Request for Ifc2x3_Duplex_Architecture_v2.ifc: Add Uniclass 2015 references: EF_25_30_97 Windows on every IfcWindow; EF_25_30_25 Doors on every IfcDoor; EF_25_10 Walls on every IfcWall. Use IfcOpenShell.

First a look at what the model holds.

```python
import ifcopenshell

model = ifcopenshell.open("Ifc2x3_Duplex_Architecture_v2.ifc")
print(model.schema)
print("classifications:", [c.Name for c in model.by_type("IfcClassification")])
for ifc_class in ("IfcDoor", "IfcRoof", "IfcStair", "IfcWall", "IfcWindow"):
    print(ifc_class, len(model.by_type(ifc_class)))
```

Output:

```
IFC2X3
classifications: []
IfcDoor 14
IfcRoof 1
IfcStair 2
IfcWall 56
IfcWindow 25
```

```python
import ifcopenshell
import ifcopenshell.api.classification

model = ifcopenshell.open("Ifc2x3_Duplex_Architecture_v2.ifc")

# IFC2X3 requires Source and Edition and has no link from the project to the system.
system = model.create_entity("IfcClassification", Source="NBS", Edition="2015", Name="Uniclass 2015")

codes = {
    "IfcWindow": ("EF_25_30_97", "Windows"),
    "IfcDoor": ("EF_25_30_25", "Doors"),
    "IfcWall": ("EF_25_10", "Walls"),
}
for ifc_class, (code, name) in codes.items():
    products = model.by_type(ifc_class)
    ifcopenshell.api.classification.add_reference(
        model, products=products, classification=system, identification=code, name=name
    )
    print(code, len(products))

model.write("Ifc2x3_Duplex_Architecture_v2_rev.ifc")
```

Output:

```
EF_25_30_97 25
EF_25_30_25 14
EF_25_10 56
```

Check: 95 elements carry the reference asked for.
